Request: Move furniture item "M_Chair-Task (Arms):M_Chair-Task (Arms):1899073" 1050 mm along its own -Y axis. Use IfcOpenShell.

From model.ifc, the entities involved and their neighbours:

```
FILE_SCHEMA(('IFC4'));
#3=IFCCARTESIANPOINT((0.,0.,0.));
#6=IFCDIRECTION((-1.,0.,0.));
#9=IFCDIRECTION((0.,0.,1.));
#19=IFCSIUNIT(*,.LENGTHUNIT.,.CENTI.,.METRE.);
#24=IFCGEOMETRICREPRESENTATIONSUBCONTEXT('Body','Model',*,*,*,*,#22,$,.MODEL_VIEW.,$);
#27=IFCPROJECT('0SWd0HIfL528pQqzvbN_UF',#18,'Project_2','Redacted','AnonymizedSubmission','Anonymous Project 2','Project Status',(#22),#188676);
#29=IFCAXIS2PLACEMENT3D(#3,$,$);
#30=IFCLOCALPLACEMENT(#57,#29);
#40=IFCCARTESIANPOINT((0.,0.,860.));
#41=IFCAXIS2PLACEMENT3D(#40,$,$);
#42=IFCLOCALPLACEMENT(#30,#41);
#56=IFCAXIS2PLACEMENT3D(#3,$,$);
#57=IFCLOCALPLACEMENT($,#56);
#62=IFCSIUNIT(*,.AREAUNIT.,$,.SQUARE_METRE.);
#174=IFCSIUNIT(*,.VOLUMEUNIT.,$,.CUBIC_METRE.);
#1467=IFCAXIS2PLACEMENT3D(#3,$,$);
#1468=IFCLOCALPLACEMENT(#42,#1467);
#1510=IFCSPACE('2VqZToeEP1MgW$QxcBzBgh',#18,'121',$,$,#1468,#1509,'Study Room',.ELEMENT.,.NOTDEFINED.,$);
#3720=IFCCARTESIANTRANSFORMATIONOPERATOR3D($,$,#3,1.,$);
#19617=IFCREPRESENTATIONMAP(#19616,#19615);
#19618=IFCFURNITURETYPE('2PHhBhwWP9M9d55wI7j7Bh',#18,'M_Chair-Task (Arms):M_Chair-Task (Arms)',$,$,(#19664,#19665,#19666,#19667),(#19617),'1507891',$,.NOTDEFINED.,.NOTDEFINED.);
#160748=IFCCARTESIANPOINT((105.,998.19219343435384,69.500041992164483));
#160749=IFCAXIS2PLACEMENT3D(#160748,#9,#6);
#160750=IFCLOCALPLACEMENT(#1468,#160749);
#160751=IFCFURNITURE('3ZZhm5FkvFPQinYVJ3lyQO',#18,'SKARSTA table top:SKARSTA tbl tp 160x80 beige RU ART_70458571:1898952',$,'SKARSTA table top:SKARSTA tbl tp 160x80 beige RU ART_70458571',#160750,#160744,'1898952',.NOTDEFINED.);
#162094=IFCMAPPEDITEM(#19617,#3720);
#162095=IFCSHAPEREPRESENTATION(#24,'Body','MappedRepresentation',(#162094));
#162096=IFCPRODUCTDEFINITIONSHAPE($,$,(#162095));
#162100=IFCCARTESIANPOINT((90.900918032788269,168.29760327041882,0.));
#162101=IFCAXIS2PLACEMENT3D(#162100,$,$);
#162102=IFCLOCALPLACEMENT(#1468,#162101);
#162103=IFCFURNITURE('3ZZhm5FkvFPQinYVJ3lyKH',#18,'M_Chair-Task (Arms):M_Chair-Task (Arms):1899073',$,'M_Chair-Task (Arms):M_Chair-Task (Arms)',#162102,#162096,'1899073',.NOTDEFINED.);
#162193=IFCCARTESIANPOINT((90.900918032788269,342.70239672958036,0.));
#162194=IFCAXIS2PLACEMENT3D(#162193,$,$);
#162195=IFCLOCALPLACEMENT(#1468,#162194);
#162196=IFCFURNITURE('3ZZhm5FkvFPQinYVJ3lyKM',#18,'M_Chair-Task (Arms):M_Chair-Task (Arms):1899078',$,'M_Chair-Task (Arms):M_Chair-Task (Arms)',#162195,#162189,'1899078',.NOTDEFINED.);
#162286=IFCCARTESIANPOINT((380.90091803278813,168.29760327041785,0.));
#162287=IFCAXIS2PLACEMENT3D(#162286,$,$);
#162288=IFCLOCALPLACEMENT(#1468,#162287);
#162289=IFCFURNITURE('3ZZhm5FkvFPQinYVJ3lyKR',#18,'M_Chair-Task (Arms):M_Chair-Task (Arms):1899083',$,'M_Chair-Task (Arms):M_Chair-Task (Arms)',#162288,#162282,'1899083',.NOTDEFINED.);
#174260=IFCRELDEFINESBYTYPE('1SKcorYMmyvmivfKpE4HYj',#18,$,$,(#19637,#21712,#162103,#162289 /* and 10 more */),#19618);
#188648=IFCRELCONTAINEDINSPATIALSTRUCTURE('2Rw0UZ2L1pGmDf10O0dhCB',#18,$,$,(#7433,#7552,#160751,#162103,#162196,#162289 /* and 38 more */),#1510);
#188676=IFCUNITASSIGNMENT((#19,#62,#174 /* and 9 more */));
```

```python
import ifcopenshell
import ifcopenshell.api.geometry
import ifcopenshell.util.placement
import ifcopenshell.util.unit

model = ifcopenshell.open("model.ifc")
unit_scale = ifcopenshell.util.unit.calculate_unit_scale(model)

item = model.by_id(162103)
matrix = ifcopenshell.util.placement.get_local_placement(item.ObjectPlacement)
matrix[:3, 3] -= matrix[:3, 1] * 1.05 / unit_scale
ifcopenshell.api.geometry.edit_object_placement(model, product=item, matrix=matrix, is_si=False)

print(ifcopenshell.util.placement.get_local_placement(item.ObjectPlacement).round(3) + 0.0)

model.write("model_edited.ifc")
```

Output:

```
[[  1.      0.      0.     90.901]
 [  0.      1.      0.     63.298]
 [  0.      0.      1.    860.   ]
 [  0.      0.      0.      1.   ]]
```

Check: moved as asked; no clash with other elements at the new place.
